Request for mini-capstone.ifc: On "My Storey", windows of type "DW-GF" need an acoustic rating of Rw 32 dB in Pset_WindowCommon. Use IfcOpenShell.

First a look at what the model holds.

```python
import ifcopenshell
import ifcopenshell.util.element

model = ifcopenshell.open("mini-capstone.ifc")
print(model.schema)
storey = next(s for s in model.by_type("IfcBuildingStorey") if s.Name == "My Storey")
windows = [e for e in ifcopenshell.util.element.get_decomposition(storey) if e.is_a("IfcWindow")]
seen = {}
for e in windows:
    element_type = ifcopenshell.util.element.get_type(e)
    key = (element_type.Name if element_type != e and element_type else None, ifcopenshell.util.element.get_pset(e, "Pset_WindowCommon", "AcousticRating"))
    seen[key] = seen.get(key, 0) + 1
for (name, value), count in sorted(seen.items(), key=str):
    print(count, "x", name, "|", value)
```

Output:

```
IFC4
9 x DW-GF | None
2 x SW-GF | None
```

```python
import ifcopenshell
import ifcopenshell.api.pset
import ifcopenshell.util.element

model = ifcopenshell.open("mini-capstone.ifc")

storey = next(s for s in model.by_type("IfcBuildingStorey") if s.Name == "My Storey")
windows = [e for e in ifcopenshell.util.element.get_decomposition(storey) if e.is_a("IfcWindow")]

count = 0
for e in windows:
    element_type = ifcopenshell.util.element.get_type(e)
    if element_type in (None, e) or element_type.Name != "DW-GF":
        continue
    # add_pset returns the element's existing set when there is one.
    pset = ifcopenshell.api.pset.add_pset(model, product=e, name="Pset_WindowCommon")
    ifcopenshell.api.pset.edit_pset(model, pset=pset, properties={"AcousticRating": "Rw 32 dB"})
    count += 1

print(count, "windows updated")

model.write("mini-capstone_rev.ifc")
```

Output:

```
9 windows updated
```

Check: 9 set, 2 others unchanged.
